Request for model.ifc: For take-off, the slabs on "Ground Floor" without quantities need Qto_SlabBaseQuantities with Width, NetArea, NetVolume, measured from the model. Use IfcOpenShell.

First a look at what the model holds.

```python
import ifcopenshell
import ifcopenshell.util.element
import ifcopenshell.util.unit

model = ifcopenshell.open("model.ifc")
print(model.schema)
for unit_type in ("LENGTHUNIT", "AREAUNIT", "VOLUMEUNIT"):
    print(unit_type, ifcopenshell.util.unit.calculate_unit_scale(model, unit_type))
storey = next(s for s in model.by_type("IfcBuildingStorey") if s.Name == "Ground Floor")
slabs = [e for e in ifcopenshell.util.element.get_decomposition(storey) if e.is_a("IfcSlab")]
for e in sorted(slabs, key=lambda e: e.id()):
    print(e.id(), e.is_a(), e.Name, list(ifcopenshell.util.element.get_psets(e, qtos_only=True)), sep=" | ")
```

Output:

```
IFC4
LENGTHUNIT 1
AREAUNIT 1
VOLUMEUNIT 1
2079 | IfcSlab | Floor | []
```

```python
import ifcopenshell
import ifcopenshell.api.pset
import ifcopenshell.geom
import ifcopenshell.util.element
import ifcopenshell.util.shape
import ifcopenshell.util.unit

model = ifcopenshell.open("model.ifc")
unit_scale = ifcopenshell.util.unit.calculate_unit_scale(model)
area_scale = ifcopenshell.util.unit.calculate_unit_scale(model, "AREAUNIT")
volume_scale = ifcopenshell.util.unit.calculate_unit_scale(model, "VOLUMEUNIT")
settings = ifcopenshell.geom.settings()

storey = next(s for s in model.by_type("IfcBuildingStorey") if s.Name == "Ground Floor")
slabs = [e for e in ifcopenshell.util.element.get_decomposition(storey) if e.is_a("IfcSlab")]

for e in sorted(slabs, key=lambda e: e.id()):
    if ifcopenshell.util.element.get_psets(e, qtos_only=True, should_inherit=False):
        continue
    # Geometry comes back in metres, in the element's own axes.
    shape = ifcopenshell.geom.create_shape(settings, e)
    values = {
        "Width": ifcopenshell.util.shape.get_z(shape.geometry) / unit_scale,
        "NetArea": ifcopenshell.util.shape.get_footprint_area(shape.geometry) / area_scale,
        "NetVolume": ifcopenshell.util.shape.get_volume(shape.geometry) / volume_scale,
    }
    qto = ifcopenshell.api.pset.add_qto(model, product=e, name="Qto_SlabBaseQuantities")
    ifcopenshell.api.pset.edit_qto(model, qto=qto, properties=values)
    print(e.id(), {k: round(v, 3) for k, v in values.items()})

model.write("model_rev.ifc")
```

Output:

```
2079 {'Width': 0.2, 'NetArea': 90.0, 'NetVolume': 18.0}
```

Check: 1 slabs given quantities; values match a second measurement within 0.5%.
